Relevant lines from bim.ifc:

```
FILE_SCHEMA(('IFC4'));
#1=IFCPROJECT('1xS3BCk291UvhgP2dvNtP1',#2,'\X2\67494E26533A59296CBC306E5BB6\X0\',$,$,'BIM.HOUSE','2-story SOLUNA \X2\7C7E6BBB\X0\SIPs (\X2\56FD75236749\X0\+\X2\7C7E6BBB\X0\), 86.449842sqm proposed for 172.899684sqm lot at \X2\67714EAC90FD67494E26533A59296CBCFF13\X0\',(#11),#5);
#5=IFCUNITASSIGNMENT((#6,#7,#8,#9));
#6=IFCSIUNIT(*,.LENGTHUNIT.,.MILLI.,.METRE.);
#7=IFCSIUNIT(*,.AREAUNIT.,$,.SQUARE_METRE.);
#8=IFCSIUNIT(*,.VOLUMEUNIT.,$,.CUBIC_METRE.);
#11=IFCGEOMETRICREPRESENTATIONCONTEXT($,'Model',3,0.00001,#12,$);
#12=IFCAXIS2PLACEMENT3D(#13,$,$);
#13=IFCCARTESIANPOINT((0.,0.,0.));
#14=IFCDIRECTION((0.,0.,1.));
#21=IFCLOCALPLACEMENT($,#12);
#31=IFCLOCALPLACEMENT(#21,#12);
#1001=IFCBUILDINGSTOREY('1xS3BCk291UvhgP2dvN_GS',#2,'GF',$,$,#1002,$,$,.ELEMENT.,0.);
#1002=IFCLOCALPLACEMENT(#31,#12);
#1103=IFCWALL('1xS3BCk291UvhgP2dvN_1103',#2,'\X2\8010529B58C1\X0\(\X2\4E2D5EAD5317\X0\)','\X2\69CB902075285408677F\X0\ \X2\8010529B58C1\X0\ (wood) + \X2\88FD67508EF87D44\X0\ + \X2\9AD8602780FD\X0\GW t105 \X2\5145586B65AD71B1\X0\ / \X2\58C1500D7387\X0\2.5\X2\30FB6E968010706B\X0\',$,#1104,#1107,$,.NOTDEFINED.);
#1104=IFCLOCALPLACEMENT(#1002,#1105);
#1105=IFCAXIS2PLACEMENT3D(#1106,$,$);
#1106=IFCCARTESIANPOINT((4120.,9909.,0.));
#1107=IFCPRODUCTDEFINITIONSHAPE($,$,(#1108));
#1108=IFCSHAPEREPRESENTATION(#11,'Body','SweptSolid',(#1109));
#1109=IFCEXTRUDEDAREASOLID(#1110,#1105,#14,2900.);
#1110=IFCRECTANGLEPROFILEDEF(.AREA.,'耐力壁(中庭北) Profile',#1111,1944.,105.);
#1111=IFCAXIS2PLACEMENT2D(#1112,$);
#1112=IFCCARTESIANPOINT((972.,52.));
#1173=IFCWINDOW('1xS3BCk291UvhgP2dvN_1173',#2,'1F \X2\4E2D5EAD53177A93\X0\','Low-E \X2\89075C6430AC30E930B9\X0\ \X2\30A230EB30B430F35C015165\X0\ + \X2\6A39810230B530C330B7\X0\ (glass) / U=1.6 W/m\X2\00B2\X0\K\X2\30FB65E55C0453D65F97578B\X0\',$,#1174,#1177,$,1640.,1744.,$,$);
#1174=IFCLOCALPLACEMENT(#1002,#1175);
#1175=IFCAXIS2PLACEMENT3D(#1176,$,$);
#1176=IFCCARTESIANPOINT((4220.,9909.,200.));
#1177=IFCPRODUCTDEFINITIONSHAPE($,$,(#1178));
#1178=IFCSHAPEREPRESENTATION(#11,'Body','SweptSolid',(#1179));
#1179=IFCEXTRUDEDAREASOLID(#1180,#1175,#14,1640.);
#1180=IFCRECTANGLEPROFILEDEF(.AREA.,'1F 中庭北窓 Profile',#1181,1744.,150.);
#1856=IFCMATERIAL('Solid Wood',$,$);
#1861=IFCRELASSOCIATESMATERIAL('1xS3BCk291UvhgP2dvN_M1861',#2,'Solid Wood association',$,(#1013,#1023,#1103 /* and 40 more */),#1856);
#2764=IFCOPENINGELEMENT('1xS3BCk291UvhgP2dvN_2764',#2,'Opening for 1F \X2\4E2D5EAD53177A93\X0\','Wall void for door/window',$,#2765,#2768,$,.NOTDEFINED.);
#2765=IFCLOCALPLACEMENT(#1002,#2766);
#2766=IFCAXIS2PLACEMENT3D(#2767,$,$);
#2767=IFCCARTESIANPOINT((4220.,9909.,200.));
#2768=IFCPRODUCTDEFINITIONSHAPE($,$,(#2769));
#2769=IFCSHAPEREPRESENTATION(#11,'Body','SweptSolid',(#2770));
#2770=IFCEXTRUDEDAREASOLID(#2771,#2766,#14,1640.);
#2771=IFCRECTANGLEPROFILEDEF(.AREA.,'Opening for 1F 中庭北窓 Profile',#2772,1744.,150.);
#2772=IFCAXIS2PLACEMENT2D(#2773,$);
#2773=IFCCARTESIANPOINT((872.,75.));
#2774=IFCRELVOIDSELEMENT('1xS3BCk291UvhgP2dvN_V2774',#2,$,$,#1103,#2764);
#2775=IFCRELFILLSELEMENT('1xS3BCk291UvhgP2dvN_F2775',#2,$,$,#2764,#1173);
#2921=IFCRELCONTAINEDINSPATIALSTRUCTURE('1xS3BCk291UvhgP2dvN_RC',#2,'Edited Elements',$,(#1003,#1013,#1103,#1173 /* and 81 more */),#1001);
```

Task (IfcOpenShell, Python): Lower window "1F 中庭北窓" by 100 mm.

```python
import numpy as np
import ifcopenshell
import ifcopenshell.api.geometry
import ifcopenshell.util.placement
import ifcopenshell.util.unit

model = ifcopenshell.open("bim.ifc")
unit_scale = ifcopenshell.util.unit.calculate_unit_scale(model)

window = model.by_guid("1xS3BCk291UvhgP2dvN_1173")
opening = window.FillsVoids[0].RelatingOpeningElement
dz = -0.1 / unit_scale

shift = np.array([0.0, 0.0, dz])
# The window is not placed relative to its opening, so move both.
for product in (opening, window):
    matrix = ifcopenshell.util.placement.get_local_placement(product.ObjectPlacement)
    matrix[:3, 3] += shift
    ifcopenshell.api.geometry.edit_object_placement(model, product=product, matrix=matrix, is_si=False)

print(f"moved by {dz * unit_scale:+.3f} m")

model.write("bim-out.ifc")
```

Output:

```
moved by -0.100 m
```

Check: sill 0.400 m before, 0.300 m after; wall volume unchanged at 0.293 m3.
